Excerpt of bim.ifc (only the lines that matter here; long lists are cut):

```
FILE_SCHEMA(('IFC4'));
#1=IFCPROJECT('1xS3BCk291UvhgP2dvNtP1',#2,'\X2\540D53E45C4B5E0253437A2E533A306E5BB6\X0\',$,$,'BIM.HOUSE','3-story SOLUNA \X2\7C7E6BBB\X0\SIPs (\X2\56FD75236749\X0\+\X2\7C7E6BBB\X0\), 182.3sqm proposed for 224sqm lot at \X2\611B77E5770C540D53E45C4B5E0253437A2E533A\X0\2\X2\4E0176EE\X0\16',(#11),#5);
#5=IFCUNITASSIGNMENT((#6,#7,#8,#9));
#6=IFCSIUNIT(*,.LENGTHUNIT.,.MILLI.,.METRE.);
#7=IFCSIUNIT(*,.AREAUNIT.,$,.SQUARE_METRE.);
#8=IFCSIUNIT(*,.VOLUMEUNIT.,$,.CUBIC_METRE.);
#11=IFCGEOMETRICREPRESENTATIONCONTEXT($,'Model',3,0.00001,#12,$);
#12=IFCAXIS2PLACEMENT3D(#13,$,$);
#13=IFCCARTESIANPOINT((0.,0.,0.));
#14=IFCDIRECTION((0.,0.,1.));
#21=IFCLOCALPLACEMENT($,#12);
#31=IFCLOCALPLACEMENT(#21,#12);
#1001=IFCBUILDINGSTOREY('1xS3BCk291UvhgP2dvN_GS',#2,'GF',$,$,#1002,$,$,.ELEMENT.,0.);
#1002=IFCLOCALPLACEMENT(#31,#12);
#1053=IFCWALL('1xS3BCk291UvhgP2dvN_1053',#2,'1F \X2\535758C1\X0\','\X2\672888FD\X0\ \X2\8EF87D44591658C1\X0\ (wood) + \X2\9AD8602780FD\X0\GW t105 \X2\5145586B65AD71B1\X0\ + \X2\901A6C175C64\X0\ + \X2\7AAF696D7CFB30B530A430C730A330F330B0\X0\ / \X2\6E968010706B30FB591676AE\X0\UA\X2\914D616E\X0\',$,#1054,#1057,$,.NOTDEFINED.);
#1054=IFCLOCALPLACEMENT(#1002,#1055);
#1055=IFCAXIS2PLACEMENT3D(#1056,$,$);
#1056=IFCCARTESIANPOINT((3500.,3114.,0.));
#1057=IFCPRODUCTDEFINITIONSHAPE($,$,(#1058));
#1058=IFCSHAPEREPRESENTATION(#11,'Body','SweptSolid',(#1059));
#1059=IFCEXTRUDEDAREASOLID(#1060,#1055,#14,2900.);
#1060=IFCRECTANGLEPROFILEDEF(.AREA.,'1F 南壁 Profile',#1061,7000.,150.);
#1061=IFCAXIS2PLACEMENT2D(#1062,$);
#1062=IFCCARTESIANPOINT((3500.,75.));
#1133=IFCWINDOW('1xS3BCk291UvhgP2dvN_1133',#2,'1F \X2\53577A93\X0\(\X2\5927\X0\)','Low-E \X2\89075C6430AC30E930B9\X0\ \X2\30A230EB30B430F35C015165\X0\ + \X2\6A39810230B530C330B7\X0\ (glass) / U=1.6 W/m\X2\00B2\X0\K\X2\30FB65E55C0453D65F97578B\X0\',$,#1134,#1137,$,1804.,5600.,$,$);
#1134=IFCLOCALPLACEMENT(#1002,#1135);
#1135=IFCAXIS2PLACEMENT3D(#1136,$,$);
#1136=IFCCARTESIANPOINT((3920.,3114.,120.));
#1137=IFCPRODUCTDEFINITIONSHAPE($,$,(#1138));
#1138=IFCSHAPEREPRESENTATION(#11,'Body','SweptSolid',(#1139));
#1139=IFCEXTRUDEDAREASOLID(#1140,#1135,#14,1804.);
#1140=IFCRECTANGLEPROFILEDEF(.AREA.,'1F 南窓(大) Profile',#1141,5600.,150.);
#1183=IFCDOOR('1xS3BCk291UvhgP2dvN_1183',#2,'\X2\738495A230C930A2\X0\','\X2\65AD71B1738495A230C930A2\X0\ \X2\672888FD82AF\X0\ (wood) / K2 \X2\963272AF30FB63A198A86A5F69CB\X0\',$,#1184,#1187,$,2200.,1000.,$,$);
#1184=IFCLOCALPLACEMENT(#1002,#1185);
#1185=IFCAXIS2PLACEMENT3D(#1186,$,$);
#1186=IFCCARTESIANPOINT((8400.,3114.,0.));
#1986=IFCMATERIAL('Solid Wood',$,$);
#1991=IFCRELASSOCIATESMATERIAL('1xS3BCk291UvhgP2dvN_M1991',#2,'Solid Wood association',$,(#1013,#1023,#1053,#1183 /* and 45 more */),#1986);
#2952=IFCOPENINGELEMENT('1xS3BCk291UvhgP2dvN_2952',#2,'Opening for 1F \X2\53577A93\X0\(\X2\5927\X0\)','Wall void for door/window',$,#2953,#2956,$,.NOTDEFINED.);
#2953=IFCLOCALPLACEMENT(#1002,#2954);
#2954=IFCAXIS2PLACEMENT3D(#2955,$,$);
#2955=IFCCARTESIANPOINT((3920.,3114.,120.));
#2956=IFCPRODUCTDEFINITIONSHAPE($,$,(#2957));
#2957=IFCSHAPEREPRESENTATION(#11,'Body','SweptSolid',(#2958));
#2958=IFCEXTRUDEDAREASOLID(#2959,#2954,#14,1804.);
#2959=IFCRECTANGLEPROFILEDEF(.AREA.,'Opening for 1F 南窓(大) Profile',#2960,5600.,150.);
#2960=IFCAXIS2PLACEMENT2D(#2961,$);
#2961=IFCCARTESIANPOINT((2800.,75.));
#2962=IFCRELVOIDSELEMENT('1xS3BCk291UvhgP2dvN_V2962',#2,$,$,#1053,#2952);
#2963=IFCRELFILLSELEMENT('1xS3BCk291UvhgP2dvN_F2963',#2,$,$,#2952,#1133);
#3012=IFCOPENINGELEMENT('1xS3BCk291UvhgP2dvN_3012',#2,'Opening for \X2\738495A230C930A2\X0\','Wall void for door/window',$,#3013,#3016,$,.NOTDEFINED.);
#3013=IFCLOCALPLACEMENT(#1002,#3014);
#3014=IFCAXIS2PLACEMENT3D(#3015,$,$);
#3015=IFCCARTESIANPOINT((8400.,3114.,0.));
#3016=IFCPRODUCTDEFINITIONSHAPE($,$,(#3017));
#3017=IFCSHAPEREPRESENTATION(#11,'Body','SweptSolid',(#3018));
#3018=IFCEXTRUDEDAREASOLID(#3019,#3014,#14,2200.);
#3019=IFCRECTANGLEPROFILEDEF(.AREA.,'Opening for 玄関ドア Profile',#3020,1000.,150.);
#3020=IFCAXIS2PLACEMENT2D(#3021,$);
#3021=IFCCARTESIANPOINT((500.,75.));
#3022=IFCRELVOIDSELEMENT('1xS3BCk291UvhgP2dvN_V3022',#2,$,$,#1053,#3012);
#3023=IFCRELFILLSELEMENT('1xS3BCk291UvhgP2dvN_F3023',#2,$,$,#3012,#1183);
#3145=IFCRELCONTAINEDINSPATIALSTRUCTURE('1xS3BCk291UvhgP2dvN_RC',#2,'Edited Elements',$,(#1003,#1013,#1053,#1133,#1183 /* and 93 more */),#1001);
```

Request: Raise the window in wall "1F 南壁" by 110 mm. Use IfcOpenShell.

```python
import numpy as np
import ifcopenshell
import ifcopenshell.api.geometry
import ifcopenshell.util.placement
import ifcopenshell.util.unit

model = ifcopenshell.open("bim.ifc")
unit_scale = ifcopenshell.util.unit.calculate_unit_scale(model)

window = model.by_id(1133)
opening = window.FillsVoids[0].RelatingOpeningElement
dz = 0.11 / unit_scale

shift = np.array([0.0, 0.0, dz])
# The window is not placed relative to its opening, so move both.
for product in (opening, window):
    matrix = ifcopenshell.util.placement.get_local_placement(product.ObjectPlacement)
    matrix[:3, 3] += shift
    ifcopenshell.api.geometry.edit_object_placement(model, product=product, matrix=matrix, is_si=False)

print(f"moved by {dz * unit_scale:+.3f} m")

model.write("bim_edited.ifc")
```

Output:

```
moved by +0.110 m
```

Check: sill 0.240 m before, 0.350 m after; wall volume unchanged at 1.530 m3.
